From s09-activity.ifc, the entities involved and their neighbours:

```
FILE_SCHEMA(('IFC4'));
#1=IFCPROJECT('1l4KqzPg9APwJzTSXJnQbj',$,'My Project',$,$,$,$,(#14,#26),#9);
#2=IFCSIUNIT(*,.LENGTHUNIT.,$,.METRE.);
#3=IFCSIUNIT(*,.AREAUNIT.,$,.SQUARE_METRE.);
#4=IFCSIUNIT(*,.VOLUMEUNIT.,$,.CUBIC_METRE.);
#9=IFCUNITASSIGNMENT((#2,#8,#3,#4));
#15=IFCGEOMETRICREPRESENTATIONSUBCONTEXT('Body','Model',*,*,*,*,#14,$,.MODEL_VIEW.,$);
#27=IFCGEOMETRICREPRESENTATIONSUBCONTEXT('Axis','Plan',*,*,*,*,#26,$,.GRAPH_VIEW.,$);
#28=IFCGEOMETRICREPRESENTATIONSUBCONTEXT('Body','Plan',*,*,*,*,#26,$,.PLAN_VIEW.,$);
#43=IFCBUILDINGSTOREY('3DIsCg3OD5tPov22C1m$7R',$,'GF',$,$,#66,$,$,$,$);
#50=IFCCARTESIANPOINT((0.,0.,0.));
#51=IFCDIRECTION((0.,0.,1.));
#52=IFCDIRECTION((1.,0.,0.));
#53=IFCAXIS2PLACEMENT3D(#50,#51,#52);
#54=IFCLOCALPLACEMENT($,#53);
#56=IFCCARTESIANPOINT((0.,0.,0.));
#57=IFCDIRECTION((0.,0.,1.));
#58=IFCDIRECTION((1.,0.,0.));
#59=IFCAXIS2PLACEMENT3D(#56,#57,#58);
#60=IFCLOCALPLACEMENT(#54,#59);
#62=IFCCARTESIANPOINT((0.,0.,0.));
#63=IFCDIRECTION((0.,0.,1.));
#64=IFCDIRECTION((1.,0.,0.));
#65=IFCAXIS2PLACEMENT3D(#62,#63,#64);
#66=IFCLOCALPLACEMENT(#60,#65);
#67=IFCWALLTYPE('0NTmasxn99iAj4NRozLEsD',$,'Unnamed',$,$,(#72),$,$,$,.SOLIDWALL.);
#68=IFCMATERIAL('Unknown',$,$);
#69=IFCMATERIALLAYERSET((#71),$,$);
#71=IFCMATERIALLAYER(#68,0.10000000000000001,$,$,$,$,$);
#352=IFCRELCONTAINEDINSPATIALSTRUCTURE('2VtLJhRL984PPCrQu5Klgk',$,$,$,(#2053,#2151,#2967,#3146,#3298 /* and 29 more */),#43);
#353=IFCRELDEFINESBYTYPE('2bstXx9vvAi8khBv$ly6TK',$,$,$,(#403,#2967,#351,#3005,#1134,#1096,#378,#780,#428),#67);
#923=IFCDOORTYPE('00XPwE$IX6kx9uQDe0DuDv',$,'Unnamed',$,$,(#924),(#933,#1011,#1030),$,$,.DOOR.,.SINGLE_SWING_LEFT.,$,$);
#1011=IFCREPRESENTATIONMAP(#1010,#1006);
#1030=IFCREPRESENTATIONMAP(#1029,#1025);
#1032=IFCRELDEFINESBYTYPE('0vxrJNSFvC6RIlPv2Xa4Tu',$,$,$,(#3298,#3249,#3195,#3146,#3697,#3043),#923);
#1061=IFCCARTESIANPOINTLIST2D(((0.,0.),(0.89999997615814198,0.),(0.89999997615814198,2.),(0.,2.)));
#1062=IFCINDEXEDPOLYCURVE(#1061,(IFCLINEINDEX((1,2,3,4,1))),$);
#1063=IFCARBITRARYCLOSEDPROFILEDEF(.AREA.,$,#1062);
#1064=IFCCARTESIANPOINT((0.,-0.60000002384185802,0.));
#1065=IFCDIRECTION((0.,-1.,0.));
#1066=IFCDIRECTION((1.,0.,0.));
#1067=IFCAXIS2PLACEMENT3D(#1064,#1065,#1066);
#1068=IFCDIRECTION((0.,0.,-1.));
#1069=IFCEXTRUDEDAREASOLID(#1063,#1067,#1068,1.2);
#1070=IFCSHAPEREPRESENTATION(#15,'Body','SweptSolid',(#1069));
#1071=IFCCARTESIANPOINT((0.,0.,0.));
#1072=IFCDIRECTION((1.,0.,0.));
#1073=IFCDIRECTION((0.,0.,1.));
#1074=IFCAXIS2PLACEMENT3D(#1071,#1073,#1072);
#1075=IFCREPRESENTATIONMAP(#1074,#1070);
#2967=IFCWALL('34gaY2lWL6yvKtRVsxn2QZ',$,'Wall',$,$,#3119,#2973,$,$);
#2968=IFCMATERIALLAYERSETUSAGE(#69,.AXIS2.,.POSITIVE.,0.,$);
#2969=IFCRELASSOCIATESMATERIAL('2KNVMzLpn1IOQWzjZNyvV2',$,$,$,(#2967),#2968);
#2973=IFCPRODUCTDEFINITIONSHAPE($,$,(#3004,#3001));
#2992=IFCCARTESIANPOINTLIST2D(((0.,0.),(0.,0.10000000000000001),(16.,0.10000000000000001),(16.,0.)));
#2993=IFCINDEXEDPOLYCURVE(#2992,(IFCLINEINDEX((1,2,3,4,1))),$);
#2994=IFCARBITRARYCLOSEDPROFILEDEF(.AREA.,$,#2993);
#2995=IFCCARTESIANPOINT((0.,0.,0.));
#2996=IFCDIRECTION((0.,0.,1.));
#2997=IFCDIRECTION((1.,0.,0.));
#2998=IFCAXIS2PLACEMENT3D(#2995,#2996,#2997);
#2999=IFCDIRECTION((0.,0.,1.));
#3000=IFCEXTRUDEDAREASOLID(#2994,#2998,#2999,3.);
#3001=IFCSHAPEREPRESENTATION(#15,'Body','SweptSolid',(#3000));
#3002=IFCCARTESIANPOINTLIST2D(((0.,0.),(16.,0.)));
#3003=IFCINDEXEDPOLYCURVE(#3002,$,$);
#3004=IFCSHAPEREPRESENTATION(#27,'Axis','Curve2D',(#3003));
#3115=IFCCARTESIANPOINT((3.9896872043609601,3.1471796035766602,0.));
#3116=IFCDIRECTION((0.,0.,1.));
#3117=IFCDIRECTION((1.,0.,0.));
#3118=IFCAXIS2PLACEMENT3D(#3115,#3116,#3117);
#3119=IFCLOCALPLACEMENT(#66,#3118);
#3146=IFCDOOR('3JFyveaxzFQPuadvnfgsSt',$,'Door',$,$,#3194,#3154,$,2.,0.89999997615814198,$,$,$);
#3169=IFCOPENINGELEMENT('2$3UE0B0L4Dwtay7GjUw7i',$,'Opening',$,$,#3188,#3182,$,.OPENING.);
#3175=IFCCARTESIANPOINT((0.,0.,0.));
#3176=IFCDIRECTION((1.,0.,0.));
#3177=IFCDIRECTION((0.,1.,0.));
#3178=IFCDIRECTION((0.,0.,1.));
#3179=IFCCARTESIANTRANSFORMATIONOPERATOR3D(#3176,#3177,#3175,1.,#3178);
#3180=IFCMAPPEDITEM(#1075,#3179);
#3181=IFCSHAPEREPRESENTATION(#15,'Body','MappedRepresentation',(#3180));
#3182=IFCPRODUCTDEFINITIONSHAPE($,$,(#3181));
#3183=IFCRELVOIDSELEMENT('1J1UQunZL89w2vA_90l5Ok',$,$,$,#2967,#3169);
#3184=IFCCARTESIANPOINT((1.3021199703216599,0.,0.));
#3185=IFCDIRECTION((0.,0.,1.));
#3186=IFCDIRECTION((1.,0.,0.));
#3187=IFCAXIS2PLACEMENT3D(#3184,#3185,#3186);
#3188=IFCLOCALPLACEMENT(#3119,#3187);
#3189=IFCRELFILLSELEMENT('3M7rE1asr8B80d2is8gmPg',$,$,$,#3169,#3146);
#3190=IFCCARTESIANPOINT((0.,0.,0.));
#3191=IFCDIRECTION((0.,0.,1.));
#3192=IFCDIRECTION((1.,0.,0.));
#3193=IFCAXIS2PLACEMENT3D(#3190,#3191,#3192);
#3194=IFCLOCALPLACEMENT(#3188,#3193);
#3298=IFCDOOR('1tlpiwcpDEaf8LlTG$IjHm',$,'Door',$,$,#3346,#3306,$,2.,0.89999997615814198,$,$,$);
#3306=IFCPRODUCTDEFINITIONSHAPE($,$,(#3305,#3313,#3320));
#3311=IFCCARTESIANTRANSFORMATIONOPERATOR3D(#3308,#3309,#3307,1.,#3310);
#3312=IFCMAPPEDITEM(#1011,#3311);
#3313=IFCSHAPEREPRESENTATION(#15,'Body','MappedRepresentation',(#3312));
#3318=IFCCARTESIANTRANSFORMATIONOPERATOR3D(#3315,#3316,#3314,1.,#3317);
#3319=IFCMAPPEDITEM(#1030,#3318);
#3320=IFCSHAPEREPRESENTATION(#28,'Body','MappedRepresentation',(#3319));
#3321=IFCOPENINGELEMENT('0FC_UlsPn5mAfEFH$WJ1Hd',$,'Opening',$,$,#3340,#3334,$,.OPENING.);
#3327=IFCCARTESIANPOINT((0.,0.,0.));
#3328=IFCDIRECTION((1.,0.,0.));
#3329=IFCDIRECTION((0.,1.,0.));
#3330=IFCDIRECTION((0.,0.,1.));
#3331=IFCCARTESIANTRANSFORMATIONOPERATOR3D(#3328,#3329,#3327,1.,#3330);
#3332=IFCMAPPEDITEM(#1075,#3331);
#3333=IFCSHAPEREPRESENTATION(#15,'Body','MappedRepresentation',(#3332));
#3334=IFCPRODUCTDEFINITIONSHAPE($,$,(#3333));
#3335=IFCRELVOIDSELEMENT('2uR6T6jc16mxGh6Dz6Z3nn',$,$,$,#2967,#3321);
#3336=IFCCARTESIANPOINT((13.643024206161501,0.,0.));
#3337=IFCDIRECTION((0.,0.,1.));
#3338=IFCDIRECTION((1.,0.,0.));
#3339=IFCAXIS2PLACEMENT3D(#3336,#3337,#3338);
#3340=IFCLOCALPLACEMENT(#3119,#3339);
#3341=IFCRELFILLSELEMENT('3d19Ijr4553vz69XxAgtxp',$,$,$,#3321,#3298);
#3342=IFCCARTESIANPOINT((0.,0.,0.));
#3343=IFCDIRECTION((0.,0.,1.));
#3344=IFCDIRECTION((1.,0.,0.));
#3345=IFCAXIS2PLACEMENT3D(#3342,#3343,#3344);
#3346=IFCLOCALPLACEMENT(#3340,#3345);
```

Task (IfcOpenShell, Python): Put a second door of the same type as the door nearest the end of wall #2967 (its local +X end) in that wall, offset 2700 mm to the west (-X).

```python
import ifcopenshell
import ifcopenshell.api.feature
import ifcopenshell.api.geometry
import ifcopenshell.api.root
import ifcopenshell.geom
import ifcopenshell.util.element
import ifcopenshell.util.placement
import ifcopenshell.util.shape
import ifcopenshell.util.unit

model = ifcopenshell.open("s09-activity.ifc")
unit_scale = ifcopenshell.util.unit.calculate_unit_scale(model)
settings = ifcopenshell.geom.settings()


def volume(element):
    """Net volume in cubic metres, openings subtracted."""
    shape = ifcopenshell.geom.create_shape(settings, element)
    return ifcopenshell.util.shape.get_volume(shape.geometry)


door = model.by_guid("1tlpiwcpDEaf8LlTG$IjHm")
opening = door.FillsVoids[0].RelatingOpeningElement
wall = opening.VoidsElements[0].RelatingBuildingElement
before = volume(wall)
shift = ifcopenshell.util.placement.get_local_placement(wall.ObjectPlacement)[:3, 0] * -2.7 / unit_scale

# copy_class copies the void relationship, type, container and properties, but no geometry.
new_opening = ifcopenshell.api.root.copy_class(model, product=opening)
new_opening.Representation = ifcopenshell.util.element.copy_deep(
    model, opening.Representation, exclude=["IfcGeometricRepresentationContext", "IfcRepresentationMap"]
)
new_door = ifcopenshell.api.root.copy_class(model, product=door)
new_door.Representation = ifcopenshell.util.element.copy_deep(
    model, door.Representation, exclude=["IfcGeometricRepresentationContext", "IfcRepresentationMap"]
)
ifcopenshell.api.feature.add_filling(model, opening=new_opening, element=new_door)

for old, new in ((opening, new_opening), (door, new_door)):
    matrix = ifcopenshell.util.placement.get_local_placement(old.ObjectPlacement)
    matrix[:3, 3] += shift
    ifcopenshell.api.geometry.edit_object_placement(model, product=new, matrix=matrix, is_si=False)

after = volume(wall)

print(f"wall volume {before:.3f} -> {after:.3f} m3")

model.write("s09-activity_v2.ifc")
```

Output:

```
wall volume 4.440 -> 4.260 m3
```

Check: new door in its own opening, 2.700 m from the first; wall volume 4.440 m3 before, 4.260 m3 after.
